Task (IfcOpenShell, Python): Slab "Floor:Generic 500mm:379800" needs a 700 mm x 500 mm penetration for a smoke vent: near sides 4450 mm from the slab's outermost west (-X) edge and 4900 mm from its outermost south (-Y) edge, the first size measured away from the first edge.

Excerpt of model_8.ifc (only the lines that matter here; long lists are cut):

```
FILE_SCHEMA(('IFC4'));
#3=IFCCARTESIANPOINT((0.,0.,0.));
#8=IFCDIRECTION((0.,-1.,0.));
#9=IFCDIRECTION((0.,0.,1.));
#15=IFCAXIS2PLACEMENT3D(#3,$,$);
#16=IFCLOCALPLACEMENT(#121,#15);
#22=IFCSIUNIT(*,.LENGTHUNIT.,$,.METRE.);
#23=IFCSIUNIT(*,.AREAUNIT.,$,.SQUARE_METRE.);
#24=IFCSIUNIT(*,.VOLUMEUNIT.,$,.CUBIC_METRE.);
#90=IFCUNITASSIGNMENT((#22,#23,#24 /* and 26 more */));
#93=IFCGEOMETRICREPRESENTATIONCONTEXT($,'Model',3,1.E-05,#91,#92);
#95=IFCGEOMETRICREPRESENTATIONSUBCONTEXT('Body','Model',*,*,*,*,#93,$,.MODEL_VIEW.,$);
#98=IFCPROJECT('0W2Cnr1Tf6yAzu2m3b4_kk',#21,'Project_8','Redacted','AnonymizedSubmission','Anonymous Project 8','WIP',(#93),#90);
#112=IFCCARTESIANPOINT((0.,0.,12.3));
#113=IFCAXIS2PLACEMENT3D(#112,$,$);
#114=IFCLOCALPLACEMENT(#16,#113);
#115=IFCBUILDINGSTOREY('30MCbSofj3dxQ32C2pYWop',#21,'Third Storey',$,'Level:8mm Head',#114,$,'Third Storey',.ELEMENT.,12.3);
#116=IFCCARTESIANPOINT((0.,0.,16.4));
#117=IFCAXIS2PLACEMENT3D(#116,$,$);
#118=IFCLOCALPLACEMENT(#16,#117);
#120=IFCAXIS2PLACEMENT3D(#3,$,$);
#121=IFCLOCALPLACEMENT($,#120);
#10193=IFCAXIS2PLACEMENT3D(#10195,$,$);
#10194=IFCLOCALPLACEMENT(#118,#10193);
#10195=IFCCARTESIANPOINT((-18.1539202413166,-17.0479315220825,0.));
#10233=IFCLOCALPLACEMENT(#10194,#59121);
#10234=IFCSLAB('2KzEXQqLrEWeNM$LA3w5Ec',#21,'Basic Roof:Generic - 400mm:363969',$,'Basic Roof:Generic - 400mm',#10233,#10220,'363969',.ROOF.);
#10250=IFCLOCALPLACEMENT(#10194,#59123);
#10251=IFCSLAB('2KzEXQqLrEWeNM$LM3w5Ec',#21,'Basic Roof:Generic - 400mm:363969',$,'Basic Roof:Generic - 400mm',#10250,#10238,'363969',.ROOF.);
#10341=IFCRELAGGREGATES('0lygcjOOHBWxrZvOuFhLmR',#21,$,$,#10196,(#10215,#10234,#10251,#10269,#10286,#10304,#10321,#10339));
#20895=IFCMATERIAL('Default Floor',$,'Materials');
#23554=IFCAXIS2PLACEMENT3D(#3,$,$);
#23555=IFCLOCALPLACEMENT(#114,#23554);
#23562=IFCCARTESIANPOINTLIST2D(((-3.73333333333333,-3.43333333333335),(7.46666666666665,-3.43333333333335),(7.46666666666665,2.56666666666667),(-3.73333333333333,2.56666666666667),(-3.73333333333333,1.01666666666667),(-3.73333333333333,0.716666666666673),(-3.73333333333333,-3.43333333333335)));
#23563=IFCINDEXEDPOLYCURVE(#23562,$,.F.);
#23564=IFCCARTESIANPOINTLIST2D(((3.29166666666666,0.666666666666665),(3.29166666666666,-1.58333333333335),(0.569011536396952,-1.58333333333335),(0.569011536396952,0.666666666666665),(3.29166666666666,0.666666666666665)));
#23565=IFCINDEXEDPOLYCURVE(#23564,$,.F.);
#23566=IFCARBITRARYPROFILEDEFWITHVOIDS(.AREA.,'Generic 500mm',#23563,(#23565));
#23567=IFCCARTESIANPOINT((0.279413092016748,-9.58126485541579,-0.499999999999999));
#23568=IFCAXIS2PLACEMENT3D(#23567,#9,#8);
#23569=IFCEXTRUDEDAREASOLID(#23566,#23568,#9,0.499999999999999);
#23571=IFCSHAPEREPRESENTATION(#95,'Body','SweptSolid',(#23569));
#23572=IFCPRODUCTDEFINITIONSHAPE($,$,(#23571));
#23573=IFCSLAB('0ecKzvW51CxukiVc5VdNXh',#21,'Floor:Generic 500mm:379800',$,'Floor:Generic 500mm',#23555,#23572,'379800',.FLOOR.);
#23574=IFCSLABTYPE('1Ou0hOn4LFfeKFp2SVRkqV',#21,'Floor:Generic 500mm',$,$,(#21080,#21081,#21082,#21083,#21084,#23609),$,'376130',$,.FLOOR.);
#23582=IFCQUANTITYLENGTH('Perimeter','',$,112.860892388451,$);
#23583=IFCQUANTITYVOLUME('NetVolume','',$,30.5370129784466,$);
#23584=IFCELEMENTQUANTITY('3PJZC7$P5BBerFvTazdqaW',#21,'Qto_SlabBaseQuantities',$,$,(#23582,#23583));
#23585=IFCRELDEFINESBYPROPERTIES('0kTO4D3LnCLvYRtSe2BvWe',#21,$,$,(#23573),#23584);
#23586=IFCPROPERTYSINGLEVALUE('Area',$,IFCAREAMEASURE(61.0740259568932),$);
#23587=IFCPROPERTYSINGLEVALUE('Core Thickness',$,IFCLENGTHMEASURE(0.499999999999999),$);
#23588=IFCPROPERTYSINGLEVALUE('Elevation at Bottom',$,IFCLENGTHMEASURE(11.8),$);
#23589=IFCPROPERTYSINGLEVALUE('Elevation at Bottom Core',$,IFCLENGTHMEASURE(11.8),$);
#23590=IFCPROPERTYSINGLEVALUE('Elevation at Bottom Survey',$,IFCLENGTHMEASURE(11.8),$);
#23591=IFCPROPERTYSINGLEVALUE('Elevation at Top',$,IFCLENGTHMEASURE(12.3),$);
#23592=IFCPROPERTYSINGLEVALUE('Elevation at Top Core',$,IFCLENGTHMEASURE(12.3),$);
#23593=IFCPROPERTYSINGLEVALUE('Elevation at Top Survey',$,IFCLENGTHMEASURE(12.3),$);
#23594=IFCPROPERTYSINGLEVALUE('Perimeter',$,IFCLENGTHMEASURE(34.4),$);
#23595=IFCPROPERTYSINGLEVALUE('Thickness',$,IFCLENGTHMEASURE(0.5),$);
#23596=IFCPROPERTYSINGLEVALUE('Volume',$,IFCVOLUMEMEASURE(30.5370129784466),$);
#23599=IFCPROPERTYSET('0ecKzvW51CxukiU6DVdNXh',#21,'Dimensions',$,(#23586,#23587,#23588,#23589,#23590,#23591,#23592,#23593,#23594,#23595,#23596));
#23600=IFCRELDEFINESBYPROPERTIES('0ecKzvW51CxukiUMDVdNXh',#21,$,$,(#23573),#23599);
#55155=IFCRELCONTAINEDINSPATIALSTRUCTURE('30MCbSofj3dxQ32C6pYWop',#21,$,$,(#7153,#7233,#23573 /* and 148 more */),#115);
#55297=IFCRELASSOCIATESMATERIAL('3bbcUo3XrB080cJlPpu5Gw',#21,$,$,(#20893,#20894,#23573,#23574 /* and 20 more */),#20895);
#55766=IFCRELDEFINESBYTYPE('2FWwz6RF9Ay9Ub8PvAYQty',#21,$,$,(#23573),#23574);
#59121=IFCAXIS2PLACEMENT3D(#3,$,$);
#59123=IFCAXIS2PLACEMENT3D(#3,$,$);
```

```python
import numpy as np
import ifcopenshell
import ifcopenshell.api.feature
import ifcopenshell.api.geometry
import ifcopenshell.api.pset
import ifcopenshell.api.root
import ifcopenshell.geom
import ifcopenshell.util.element
import ifcopenshell.util.placement
import ifcopenshell.util.representation
import ifcopenshell.util.shape
import ifcopenshell.util.unit

model = ifcopenshell.open("model_8.ifc")
unit_scale = ifcopenshell.util.unit.calculate_unit_scale(model)
area_scale = ifcopenshell.util.unit.calculate_unit_scale(model, "AREAUNIT")
volume_scale = ifcopenshell.util.unit.calculate_unit_scale(model, "VOLUMEUNIT")
settings = ifcopenshell.geom.settings()


def volume(element):
    """Net volume in cubic metres, openings subtracted."""
    shape = ifcopenshell.geom.create_shape(settings, element)
    return ifcopenshell.util.shape.get_volume(shape.geometry)


slab = model.by_guid("0ecKzvW51CxukiVc5VdNXh")
before = volume(slab)

# Extent in the slab's own axes, in metres. The edges named are its -X and -Y sides.
slab_shape = ifcopenshell.geom.create_shape(settings, slab)
vertices = ifcopenshell.util.shape.get_vertices(slab_shape.geometry)
x_min, y_min, bottom = vertices.min(axis=0)
top = vertices[:, 2].max()

opening = ifcopenshell.api.root.create_entity(model, ifc_class="IfcOpeningElement", name="Smoke vent opening", predefined_type="OPENING")
context = ifcopenshell.util.representation.get_context(model, "Model", "Body", "MODEL_VIEW")
width, depth = 0.7, 0.5
outline = [(0.0, 0.0), (width, 0.0), (width, depth), (0.0, depth), (0.0, 0.0)]
# Overshoot both faces by 50 mm so the cut is clean.
shape = ifcopenshell.api.geometry.add_slab_representation(
    model, context=context, depth=top - bottom + 0.1, polyline=outline
)
ifcopenshell.api.geometry.assign_representation(model, product=opening, representation=shape)

matrix = ifcopenshell.util.placement.get_local_placement(slab.ObjectPlacement)
matrix[:, 3] = matrix @ np.append(np.array([x_min + 4.45, y_min + 4.9, bottom - 0.05]) / unit_scale, 1.0)
ifcopenshell.api.geometry.edit_object_placement(model, product=opening, matrix=matrix, is_si=False)
ifcopenshell.api.feature.add_feature(model, feature=opening, element=slab)

after = volume(slab)

# Update the slab's stored quantities.
qto = model.by_id(ifcopenshell.util.element.get_pset(slab, "Qto_SlabBaseQuantities", should_inherit=False)["id"])
ifcopenshell.api.pset.edit_qto(model, qto=qto, properties={"NetVolume": after / volume_scale})
pset = model.by_id(ifcopenshell.util.element.get_pset(slab, "Dimensions", should_inherit=False)["id"])
ifcopenshell.api.pset.edit_pset(model, pset=pset, properties={
    "Area": model.create_entity("IfcAreaMeasure", after / (top - bottom) / area_scale),
    "Volume": model.create_entity("IfcVolumeMeasure", after / volume_scale),
})

print(f"slab volume {before:.3f} -> {after:.3f} m3")

model.write("model_8-out.ifc")
```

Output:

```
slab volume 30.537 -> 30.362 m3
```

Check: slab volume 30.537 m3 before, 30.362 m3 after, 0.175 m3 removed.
